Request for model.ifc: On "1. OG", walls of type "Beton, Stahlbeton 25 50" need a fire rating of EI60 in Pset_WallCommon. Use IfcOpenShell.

First a look at what the model holds.

```python
import ifcopenshell
import ifcopenshell.util.element

model = ifcopenshell.open("model.ifc")
print(model.schema)
storey = next(s for s in model.by_type("IfcBuildingStorey") if s.Name == "1. OG")
walls = [e for e in ifcopenshell.util.element.get_decomposition(storey) if e.is_a("IfcWall")]
seen = {}
for e in walls:
    element_type = ifcopenshell.util.element.get_type(e)
    key = (element_type.Name if element_type != e and element_type else None, ifcopenshell.util.element.get_pset(e, "Pset_WallCommon", "FireRating"))
    seen[key] = seen.get(key, 0) + 1
for (name, value), count in sorted(seen.items(), key=str):
    print(count, "x", name, "|", value)
```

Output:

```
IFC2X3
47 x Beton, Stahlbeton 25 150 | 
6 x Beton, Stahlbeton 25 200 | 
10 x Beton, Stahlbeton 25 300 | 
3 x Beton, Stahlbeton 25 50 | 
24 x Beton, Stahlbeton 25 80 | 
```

```python
import ifcopenshell
import ifcopenshell.api.pset
import ifcopenshell.util.element

model = ifcopenshell.open("model.ifc")

storey = next(s for s in model.by_type("IfcBuildingStorey") if s.Name == "1. OG")
walls = [e for e in ifcopenshell.util.element.get_decomposition(storey) if e.is_a("IfcWall")]

count = 0
for e in walls:
    element_type = ifcopenshell.util.element.get_type(e)
    if element_type in (None, e) or element_type.Name != "Beton, Stahlbeton 25 50":
        continue
    # add_pset returns the element's existing set when there is one.
    pset = ifcopenshell.api.pset.add_pset(model, product=e, name="Pset_WallCommon")
    ifcopenshell.api.pset.edit_pset(model, pset=pset, properties={"FireRating": "EI60"})
    count += 1

print(count, "walls updated")

model.write("model-out.ifc")
```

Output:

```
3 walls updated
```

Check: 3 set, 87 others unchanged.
